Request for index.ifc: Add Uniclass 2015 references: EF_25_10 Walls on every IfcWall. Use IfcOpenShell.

First a look at what the model holds.

```python
import ifcopenshell

model = ifcopenshell.open("index.ifc")
print(model.schema)
print("classifications:", [c.Name for c in model.by_type("IfcClassification")])
for ifc_class in ("IfcDoor", "IfcRoof", "IfcStair", "IfcWall", "IfcWindow"):
    print(ifc_class, len(model.by_type(ifc_class)))
```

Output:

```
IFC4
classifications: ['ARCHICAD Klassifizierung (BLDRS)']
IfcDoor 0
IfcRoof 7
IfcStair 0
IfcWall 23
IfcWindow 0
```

```python
import ifcopenshell
import ifcopenshell.api.classification

model = ifcopenshell.open("index.ifc")

system = ifcopenshell.api.classification.add_classification(model, classification="Uniclass 2015")

codes = {
    "IfcWall": ("EF_25_10", "Walls"),
}
for ifc_class, (code, name) in codes.items():
    products = model.by_type(ifc_class)
    ifcopenshell.api.classification.add_reference(
        model, products=products, classification=system, identification=code, name=name
    )
    print(code, len(products))

model.write("index_rev.ifc")
```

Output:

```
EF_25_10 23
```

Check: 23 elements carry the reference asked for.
